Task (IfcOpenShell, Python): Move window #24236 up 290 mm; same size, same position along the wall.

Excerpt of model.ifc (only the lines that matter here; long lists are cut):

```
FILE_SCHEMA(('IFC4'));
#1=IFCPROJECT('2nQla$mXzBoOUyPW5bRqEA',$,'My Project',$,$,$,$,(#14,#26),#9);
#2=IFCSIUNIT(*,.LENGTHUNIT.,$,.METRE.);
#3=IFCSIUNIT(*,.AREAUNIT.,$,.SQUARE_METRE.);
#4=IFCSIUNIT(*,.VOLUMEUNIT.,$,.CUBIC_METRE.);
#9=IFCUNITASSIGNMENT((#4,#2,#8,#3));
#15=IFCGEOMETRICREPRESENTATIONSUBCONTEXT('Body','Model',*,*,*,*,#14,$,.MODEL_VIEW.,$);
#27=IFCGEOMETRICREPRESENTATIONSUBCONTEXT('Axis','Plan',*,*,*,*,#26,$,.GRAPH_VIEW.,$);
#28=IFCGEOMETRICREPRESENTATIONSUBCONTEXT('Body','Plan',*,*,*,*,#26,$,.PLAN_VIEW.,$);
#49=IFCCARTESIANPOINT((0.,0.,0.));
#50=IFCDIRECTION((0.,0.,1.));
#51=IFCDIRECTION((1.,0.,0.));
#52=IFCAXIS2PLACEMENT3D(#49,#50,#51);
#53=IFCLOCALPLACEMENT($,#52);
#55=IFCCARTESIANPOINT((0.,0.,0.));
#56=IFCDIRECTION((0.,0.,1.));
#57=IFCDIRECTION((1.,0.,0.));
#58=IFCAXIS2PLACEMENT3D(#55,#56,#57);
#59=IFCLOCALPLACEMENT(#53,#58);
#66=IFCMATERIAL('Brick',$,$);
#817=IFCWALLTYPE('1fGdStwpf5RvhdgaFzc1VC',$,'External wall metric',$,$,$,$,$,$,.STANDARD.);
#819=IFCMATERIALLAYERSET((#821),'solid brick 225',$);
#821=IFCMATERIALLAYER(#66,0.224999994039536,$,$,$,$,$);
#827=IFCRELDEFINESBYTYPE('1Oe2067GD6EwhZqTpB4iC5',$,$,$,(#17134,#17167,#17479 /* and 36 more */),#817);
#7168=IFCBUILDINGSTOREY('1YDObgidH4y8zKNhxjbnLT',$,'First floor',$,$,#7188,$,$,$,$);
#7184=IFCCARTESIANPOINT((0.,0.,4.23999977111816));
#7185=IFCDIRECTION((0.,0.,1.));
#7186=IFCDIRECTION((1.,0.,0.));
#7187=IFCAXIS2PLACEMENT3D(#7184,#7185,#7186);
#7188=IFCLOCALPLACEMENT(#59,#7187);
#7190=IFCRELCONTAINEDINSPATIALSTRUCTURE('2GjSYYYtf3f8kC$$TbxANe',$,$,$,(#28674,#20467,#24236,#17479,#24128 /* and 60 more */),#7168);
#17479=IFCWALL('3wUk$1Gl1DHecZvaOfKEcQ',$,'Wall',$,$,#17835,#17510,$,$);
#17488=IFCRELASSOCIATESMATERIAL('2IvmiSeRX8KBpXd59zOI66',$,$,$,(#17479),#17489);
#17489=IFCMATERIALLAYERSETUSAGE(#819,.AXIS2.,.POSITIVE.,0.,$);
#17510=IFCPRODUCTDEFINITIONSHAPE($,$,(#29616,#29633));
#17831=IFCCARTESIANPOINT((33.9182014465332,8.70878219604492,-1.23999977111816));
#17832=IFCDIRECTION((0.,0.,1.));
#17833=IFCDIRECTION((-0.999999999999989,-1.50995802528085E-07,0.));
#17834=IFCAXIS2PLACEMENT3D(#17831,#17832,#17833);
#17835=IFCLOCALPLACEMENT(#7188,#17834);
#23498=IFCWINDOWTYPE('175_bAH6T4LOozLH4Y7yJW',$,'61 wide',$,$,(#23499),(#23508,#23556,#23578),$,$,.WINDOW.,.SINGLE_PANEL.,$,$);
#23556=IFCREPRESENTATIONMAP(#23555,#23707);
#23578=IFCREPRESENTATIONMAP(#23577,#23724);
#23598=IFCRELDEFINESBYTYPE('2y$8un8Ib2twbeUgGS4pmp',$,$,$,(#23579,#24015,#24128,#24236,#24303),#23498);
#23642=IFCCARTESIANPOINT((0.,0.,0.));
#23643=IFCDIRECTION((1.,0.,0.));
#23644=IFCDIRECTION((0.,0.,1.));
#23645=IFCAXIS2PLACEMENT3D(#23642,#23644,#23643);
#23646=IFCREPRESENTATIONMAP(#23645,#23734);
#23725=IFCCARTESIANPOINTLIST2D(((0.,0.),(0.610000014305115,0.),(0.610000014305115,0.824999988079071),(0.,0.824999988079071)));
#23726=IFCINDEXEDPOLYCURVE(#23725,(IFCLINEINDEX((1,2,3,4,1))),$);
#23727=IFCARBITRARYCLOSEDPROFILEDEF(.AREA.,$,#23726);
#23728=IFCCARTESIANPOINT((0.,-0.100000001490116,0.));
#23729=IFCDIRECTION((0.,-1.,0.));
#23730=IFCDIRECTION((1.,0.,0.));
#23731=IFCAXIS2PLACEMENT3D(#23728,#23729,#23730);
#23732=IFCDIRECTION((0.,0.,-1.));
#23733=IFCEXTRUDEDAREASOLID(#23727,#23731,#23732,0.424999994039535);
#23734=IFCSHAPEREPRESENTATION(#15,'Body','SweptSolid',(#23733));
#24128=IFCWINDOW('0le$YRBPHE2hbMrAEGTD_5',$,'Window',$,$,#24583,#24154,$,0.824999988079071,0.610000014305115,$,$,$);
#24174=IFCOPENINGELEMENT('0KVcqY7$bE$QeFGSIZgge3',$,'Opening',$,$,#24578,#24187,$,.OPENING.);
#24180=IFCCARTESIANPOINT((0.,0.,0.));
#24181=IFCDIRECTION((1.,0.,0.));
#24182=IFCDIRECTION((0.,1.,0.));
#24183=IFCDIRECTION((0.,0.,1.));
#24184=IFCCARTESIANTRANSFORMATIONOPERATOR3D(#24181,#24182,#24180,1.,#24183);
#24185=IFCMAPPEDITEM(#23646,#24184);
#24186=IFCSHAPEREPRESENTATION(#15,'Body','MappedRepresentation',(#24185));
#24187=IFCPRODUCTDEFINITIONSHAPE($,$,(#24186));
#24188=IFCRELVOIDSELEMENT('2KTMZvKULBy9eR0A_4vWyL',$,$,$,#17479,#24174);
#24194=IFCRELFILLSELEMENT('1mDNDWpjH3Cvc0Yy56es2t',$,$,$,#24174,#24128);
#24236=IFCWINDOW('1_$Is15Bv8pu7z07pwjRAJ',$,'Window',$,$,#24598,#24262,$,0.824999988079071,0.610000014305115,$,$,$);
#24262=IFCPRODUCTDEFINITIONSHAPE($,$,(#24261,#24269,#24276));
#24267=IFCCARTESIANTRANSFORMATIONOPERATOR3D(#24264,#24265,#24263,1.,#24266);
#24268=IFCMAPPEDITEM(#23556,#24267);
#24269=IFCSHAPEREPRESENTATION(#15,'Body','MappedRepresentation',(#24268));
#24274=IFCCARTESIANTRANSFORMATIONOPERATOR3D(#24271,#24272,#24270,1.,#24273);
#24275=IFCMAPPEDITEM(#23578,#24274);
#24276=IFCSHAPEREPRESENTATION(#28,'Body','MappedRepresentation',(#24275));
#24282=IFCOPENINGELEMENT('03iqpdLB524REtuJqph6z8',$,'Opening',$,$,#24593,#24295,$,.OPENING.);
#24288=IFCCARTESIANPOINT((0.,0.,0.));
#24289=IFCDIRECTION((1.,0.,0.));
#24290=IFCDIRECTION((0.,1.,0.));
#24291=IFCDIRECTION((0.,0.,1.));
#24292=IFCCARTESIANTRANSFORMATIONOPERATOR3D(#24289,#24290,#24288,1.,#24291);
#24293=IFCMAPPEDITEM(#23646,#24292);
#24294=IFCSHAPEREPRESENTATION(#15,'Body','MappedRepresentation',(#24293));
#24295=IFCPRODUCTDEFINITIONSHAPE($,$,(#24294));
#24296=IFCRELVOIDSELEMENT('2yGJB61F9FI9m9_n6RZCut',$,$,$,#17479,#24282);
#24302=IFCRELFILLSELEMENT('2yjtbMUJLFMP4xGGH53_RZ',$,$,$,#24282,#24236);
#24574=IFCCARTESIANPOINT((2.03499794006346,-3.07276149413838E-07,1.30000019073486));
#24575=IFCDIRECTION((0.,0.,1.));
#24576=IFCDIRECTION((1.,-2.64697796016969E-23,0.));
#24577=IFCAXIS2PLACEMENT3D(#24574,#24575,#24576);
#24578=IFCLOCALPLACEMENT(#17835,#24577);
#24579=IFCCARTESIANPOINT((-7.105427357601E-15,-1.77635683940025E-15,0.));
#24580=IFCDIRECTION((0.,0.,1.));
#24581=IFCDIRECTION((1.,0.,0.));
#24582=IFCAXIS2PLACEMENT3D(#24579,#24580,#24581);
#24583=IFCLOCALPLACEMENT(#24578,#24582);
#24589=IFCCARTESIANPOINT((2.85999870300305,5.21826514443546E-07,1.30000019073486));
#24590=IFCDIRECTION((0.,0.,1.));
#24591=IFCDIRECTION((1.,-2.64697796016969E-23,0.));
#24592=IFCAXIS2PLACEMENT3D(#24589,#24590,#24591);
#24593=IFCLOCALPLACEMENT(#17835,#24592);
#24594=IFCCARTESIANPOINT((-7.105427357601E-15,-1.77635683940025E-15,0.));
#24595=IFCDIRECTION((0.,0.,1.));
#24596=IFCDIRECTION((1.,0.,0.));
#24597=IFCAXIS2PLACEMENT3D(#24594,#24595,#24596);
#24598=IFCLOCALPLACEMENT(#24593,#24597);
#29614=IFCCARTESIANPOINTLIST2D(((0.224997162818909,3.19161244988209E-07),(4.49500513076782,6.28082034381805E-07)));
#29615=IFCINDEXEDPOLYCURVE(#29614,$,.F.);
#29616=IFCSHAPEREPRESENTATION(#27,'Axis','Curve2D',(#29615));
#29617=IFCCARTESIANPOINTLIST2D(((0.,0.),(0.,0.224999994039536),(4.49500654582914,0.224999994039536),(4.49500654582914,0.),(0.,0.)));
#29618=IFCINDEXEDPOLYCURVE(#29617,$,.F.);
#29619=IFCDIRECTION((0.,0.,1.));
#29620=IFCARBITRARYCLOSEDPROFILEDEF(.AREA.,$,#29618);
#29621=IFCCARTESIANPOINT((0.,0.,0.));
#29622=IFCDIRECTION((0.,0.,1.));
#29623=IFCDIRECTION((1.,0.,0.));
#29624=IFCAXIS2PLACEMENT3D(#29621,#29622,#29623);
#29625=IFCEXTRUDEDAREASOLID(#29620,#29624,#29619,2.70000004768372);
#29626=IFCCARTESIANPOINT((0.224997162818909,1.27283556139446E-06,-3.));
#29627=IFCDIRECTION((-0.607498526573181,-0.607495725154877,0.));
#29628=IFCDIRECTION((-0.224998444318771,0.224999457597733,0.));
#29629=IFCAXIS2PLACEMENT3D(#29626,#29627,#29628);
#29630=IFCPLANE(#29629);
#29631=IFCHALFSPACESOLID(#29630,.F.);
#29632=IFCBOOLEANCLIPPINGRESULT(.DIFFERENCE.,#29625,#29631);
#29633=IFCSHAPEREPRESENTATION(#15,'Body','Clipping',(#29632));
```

```python
import numpy as np
import ifcopenshell
import ifcopenshell.api.geometry
import ifcopenshell.util.placement
import ifcopenshell.util.unit

model = ifcopenshell.open("model.ifc")
unit_scale = ifcopenshell.util.unit.calculate_unit_scale(model)

window = model.by_id(24236)
opening = window.FillsVoids[0].RelatingOpeningElement
dz = 0.29 / unit_scale

shift = np.array([0.0, 0.0, dz])
# The window is placed relative to its opening, so it follows when the opening moves.
matrix = ifcopenshell.util.placement.get_local_placement(opening.ObjectPlacement)
matrix[:3, 3] += shift
ifcopenshell.api.geometry.edit_object_placement(
    model, product=opening, matrix=matrix, is_si=False, should_transform_children=True
)

print(f"moved by {dz * unit_scale:+.3f} m")

model.write("model_updated.ifc")
```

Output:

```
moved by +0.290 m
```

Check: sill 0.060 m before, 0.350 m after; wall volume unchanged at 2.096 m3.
